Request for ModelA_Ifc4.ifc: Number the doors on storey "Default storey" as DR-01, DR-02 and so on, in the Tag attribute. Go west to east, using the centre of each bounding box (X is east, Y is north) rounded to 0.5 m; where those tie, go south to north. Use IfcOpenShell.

First a look at what the model holds.

```python
import ifcopenshell
import ifcopenshell.util.element
import ifcopenshell.util.placement

model = ifcopenshell.open("ModelA_Ifc4.ifc")
print(model.schema)
storey = next(s for s in model.by_type("IfcBuildingStorey") if s.Name == "Default storey")
doors = [e for e in ifcopenshell.util.element.get_decomposition(storey) if e.is_a("IfcDoor")]
for e in sorted(doors, key=lambda e: e.id()):
    origin = ifcopenshell.util.placement.get_local_placement(e.ObjectPlacement)[:3, 3]
    print(e.id(), e.Tag, e.Name, origin.round(2) + 0.0, sep=" | ")
```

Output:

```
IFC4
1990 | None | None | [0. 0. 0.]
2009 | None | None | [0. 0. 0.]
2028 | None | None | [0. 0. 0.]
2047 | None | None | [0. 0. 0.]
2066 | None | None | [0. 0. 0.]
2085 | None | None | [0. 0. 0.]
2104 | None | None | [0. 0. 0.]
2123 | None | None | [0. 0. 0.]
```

```python
import ifcopenshell
import ifcopenshell.geom
import ifcopenshell.util.element
import ifcopenshell.util.shape

model = ifcopenshell.open("ModelA_Ifc4.ifc")
settings = ifcopenshell.geom.settings()
settings.set("use-world-coords", True)


def centre(element):
    shape = ifcopenshell.geom.create_shape(settings, element)
    return ifcopenshell.util.shape.get_bbox_centroid(shape.geometry)


storey = next(s for s in model.by_type("IfcBuildingStorey") if s.Name == "Default storey")
doors = [e for e in ifcopenshell.util.element.get_decomposition(storey) if e.is_a("IfcDoor")]

# Insertion points can sit at a corner or the storey origin, so sort by the geometry (in metres).
centres = {e: centre(e) for e in doors}
doors.sort(key=lambda e: (round(centres[e][0] / 0.5), centres[e][1]))

for i, e in enumerate(doors, start=1):
    number = f"DR-{i:02d}"
    e.Tag = number
    print(e.id(), number)

model.write("ModelA_Ifc4_edited.ifc")
```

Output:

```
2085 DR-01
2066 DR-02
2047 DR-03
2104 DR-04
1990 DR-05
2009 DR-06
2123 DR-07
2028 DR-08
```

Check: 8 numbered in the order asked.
